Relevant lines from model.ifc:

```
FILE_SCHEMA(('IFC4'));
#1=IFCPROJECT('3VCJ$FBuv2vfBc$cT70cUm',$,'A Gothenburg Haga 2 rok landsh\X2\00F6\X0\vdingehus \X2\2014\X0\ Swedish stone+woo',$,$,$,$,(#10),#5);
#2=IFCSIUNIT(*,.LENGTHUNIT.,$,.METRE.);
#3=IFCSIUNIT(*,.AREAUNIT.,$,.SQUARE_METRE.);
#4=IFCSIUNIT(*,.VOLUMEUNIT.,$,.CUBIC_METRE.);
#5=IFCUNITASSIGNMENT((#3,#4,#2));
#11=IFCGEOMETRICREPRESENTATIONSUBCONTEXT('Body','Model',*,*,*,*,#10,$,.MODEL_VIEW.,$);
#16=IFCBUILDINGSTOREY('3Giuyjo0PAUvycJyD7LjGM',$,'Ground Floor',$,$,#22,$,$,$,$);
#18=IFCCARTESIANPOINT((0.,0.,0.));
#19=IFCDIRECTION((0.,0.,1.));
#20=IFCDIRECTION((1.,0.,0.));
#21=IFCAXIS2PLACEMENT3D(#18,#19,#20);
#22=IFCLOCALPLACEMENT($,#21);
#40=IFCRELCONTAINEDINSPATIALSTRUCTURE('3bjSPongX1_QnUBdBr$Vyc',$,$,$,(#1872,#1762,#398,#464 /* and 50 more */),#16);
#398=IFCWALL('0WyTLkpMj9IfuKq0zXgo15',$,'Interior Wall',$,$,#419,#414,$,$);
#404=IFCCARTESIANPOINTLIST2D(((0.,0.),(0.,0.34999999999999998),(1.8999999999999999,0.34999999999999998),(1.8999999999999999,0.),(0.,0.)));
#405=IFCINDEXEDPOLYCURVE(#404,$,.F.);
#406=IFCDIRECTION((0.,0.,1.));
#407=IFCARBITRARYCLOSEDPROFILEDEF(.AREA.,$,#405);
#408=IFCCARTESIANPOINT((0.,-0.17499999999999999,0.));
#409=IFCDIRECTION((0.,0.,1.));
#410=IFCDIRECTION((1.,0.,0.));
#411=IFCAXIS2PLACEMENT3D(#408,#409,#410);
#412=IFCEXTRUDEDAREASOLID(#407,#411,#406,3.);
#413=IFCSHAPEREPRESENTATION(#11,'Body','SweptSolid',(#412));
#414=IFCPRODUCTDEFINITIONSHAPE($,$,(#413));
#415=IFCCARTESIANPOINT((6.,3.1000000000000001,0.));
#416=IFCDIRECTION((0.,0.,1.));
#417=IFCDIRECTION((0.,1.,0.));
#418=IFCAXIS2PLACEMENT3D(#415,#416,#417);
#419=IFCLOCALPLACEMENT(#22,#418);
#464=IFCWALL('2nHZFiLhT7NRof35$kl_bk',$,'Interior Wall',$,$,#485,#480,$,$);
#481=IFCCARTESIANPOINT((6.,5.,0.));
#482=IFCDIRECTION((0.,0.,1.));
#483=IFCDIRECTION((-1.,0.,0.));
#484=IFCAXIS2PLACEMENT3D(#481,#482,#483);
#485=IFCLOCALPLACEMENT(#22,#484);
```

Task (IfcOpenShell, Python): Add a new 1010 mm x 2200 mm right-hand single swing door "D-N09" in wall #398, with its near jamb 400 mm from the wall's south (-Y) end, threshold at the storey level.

```python
import numpy as np
import ifcopenshell
import ifcopenshell.api.feature
import ifcopenshell.api.geometry
import ifcopenshell.api.root
import ifcopenshell.api.spatial
import ifcopenshell.geom
import ifcopenshell.util.element
import ifcopenshell.util.placement
import ifcopenshell.util.representation
import ifcopenshell.util.shape
import ifcopenshell.util.unit

model = ifcopenshell.open("model.ifc")
unit_scale = ifcopenshell.util.unit.calculate_unit_scale(model)
settings = ifcopenshell.geom.settings()


def volume(element):
    """Net volume in cubic metres, openings subtracted."""
    shape = ifcopenshell.geom.create_shape(settings, element)
    return ifcopenshell.util.shape.get_volume(shape.geometry)


wall = model.by_id(398)
storey = ifcopenshell.util.element.get_container(wall, ifc_class="IfcBuildingStorey")
context = ifcopenshell.util.representation.get_context(model, "Model", "Body", "MODEL_VIEW")
before = volume(wall)

width, height, from_end, sill = 1.01, 2.2, 0.4, 0.0  # metres

# The wall runs along its own X axis, and the end named is its -X end.
wall_shape = ifcopenshell.geom.create_shape(settings, wall)
x, y, z = ifcopenshell.util.shape.get_vertices(wall_shape.geometry).T
start = x.min() + from_end
face, thickness = float(y.min()), float(y.max() - y.min())
wall_matrix = ifcopenshell.util.placement.get_local_placement(wall.ObjectPlacement)
level = ifcopenshell.util.placement.get_local_placement(storey.ObjectPlacement)[2, 3]


def in_wall(x, y):
    """Placement at x, y metres in the wall's axes, at sill height."""
    matrix = wall_matrix.copy()
    matrix[:, 3] = wall_matrix @ np.array([x / unit_scale, y / unit_scale, 0.0, 1.0])
    matrix[2, 3] = level + sill / unit_scale
    return matrix


# Opening: a box that overshoots both wall faces by 50 mm.
opening = ifcopenshell.api.root.create_entity(model, ifc_class="IfcOpeningElement", predefined_type="OPENING")
box = ifcopenshell.api.geometry.add_wall_representation(
    model, context=context, length=width, height=height, thickness=thickness + 0.1
)
ifcopenshell.api.geometry.assign_representation(model, product=opening, representation=box)
ifcopenshell.api.geometry.edit_object_placement(model, product=opening, matrix=in_wall(start, face - 0.05), is_si=False)
ifcopenshell.api.feature.add_feature(model, feature=opening, element=wall)

door = ifcopenshell.api.root.create_entity(model, ifc_class="IfcDoor", name="D-N09", predefined_type="DOOR")
door.OverallWidth, door.OverallHeight = width / unit_scale, height / unit_scale
door.OperationType = "SINGLE_SWING_RIGHT"
body = ifcopenshell.api.geometry.add_door_representation(
    model,
    context=context,
    overall_width=door.OverallWidth,
    overall_height=door.OverallHeight,
    operation_type="SINGLE_SWING_RIGHT",
    lining_properties={"LiningDepth": thickness / unit_scale, "ThresholdDepth": thickness / unit_scale},
)
ifcopenshell.api.geometry.assign_representation(model, product=door, representation=body)
ifcopenshell.api.spatial.assign_container(model, products=[door], relating_structure=storey)
ifcopenshell.api.feature.add_filling(model, opening=opening, element=door)

# The lining spans the wall, so the door starts at the wall face.
ifcopenshell.api.geometry.edit_object_placement(model, product=door, matrix=in_wall(start, face), is_si=False)

after = volume(wall)

print(f"wall volume {before:.3f} -> {after:.3f} m3")

model.write("model_v2.ifc")
```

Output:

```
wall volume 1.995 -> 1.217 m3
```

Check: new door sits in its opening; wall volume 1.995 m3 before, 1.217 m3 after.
